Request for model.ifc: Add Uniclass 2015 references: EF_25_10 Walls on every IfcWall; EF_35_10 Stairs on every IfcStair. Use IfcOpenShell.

First a look at what the model holds.

```python
import ifcopenshell

model = ifcopenshell.open("model.ifc")
print(model.schema)
print("classifications:", [c.Name for c in model.by_type("IfcClassification")])
for ifc_class in ("IfcDoor", "IfcRoof", "IfcStair", "IfcWall", "IfcWindow"):
    print(ifc_class, len(model.by_type(ifc_class)))
```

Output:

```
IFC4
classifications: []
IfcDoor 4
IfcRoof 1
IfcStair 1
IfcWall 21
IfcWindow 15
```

```python
import ifcopenshell
import ifcopenshell.api.classification

model = ifcopenshell.open("model.ifc")

system = ifcopenshell.api.classification.add_classification(model, classification="Uniclass 2015")

codes = {
    "IfcWall": ("EF_25_10", "Walls"),
    "IfcStair": ("EF_35_10", "Stairs"),
}
for ifc_class, (code, name) in codes.items():
    products = model.by_type(ifc_class)
    ifcopenshell.api.classification.add_reference(
        model, products=products, classification=system, identification=code, name=name
    )
    print(code, len(products))

model.write("model_edited.ifc")
```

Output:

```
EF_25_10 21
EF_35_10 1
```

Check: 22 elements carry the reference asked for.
